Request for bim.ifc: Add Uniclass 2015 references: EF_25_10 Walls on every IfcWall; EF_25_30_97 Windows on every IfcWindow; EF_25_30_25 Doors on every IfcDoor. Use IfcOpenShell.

First a look at what the model holds.

```python
import ifcopenshell

model = ifcopenshell.open("bim.ifc")
print(model.schema)
print("classifications:", [c.Name for c in model.by_type("IfcClassification")])
for ifc_class in ("IfcDoor", "IfcRoof", "IfcStair", "IfcWall", "IfcWindow"):
    print(ifc_class, len(model.by_type(ifc_class)))
```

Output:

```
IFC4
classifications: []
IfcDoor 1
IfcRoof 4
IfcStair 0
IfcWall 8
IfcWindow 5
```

```python
import ifcopenshell
import ifcopenshell.api.classification

model = ifcopenshell.open("bim.ifc")

system = ifcopenshell.api.classification.add_classification(model, classification="Uniclass 2015")

codes = {
    "IfcWall": ("EF_25_10", "Walls"),
    "IfcWindow": ("EF_25_30_97", "Windows"),
    "IfcDoor": ("EF_25_30_25", "Doors"),
}
for ifc_class, (code, name) in codes.items():
    products = model.by_type(ifc_class)
    ifcopenshell.api.classification.add_reference(
        model, products=products, classification=system, identification=code, name=name
    )
    print(code, len(products))

model.write("bim_rev.ifc")
```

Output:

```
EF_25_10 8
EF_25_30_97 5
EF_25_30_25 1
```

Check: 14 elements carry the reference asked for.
